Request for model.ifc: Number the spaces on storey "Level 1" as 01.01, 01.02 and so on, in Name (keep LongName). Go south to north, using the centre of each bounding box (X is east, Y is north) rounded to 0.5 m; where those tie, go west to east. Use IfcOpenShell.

First a look at what the model holds.

```python
import ifcopenshell
import ifcopenshell.util.element
import ifcopenshell.util.placement

model = ifcopenshell.open("model.ifc")
print(model.schema)
storey = next(s for s in model.by_type("IfcBuildingStorey") if s.Name == "Level 1")
spaces = [e for e in ifcopenshell.util.element.get_decomposition(storey) if e.is_a("IfcSpace")]
for e in sorted(spaces, key=lambda e: e.id()):
    origin = ifcopenshell.util.placement.get_local_placement(e.ObjectPlacement)[:3, 3]
    print(e.id(), e.Name, e.LongName, origin.round(2) + 0.0, sep=" | ")
```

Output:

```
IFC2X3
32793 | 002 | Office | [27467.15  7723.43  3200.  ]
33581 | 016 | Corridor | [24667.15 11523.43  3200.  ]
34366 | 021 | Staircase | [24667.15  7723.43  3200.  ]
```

```python
import ifcopenshell
import ifcopenshell.geom
import ifcopenshell.util.element
import ifcopenshell.util.shape

model = ifcopenshell.open("model.ifc")
settings = ifcopenshell.geom.settings()
settings.set("use-world-coords", True)


def centre(element):
    shape = ifcopenshell.geom.create_shape(settings, element)
    return ifcopenshell.util.shape.get_bbox_centroid(shape.geometry)


storey = next(s for s in model.by_type("IfcBuildingStorey") if s.Name == "Level 1")
spaces = [e for e in ifcopenshell.util.element.get_decomposition(storey) if e.is_a("IfcSpace")]

# Insertion points can sit at a corner or the storey origin, so sort by the geometry (in metres).
centres = {e: centre(e) for e in spaces}
spaces.sort(key=lambda e: (round(centres[e][1] / 0.5), centres[e][0]))

for i, e in enumerate(spaces, start=1):
    number = f"01.{i:02d}"
    e.Name = number
    print(e.id(), number)

model.write("model_v2.ifc")
```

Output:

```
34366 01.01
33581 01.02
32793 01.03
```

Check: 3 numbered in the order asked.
